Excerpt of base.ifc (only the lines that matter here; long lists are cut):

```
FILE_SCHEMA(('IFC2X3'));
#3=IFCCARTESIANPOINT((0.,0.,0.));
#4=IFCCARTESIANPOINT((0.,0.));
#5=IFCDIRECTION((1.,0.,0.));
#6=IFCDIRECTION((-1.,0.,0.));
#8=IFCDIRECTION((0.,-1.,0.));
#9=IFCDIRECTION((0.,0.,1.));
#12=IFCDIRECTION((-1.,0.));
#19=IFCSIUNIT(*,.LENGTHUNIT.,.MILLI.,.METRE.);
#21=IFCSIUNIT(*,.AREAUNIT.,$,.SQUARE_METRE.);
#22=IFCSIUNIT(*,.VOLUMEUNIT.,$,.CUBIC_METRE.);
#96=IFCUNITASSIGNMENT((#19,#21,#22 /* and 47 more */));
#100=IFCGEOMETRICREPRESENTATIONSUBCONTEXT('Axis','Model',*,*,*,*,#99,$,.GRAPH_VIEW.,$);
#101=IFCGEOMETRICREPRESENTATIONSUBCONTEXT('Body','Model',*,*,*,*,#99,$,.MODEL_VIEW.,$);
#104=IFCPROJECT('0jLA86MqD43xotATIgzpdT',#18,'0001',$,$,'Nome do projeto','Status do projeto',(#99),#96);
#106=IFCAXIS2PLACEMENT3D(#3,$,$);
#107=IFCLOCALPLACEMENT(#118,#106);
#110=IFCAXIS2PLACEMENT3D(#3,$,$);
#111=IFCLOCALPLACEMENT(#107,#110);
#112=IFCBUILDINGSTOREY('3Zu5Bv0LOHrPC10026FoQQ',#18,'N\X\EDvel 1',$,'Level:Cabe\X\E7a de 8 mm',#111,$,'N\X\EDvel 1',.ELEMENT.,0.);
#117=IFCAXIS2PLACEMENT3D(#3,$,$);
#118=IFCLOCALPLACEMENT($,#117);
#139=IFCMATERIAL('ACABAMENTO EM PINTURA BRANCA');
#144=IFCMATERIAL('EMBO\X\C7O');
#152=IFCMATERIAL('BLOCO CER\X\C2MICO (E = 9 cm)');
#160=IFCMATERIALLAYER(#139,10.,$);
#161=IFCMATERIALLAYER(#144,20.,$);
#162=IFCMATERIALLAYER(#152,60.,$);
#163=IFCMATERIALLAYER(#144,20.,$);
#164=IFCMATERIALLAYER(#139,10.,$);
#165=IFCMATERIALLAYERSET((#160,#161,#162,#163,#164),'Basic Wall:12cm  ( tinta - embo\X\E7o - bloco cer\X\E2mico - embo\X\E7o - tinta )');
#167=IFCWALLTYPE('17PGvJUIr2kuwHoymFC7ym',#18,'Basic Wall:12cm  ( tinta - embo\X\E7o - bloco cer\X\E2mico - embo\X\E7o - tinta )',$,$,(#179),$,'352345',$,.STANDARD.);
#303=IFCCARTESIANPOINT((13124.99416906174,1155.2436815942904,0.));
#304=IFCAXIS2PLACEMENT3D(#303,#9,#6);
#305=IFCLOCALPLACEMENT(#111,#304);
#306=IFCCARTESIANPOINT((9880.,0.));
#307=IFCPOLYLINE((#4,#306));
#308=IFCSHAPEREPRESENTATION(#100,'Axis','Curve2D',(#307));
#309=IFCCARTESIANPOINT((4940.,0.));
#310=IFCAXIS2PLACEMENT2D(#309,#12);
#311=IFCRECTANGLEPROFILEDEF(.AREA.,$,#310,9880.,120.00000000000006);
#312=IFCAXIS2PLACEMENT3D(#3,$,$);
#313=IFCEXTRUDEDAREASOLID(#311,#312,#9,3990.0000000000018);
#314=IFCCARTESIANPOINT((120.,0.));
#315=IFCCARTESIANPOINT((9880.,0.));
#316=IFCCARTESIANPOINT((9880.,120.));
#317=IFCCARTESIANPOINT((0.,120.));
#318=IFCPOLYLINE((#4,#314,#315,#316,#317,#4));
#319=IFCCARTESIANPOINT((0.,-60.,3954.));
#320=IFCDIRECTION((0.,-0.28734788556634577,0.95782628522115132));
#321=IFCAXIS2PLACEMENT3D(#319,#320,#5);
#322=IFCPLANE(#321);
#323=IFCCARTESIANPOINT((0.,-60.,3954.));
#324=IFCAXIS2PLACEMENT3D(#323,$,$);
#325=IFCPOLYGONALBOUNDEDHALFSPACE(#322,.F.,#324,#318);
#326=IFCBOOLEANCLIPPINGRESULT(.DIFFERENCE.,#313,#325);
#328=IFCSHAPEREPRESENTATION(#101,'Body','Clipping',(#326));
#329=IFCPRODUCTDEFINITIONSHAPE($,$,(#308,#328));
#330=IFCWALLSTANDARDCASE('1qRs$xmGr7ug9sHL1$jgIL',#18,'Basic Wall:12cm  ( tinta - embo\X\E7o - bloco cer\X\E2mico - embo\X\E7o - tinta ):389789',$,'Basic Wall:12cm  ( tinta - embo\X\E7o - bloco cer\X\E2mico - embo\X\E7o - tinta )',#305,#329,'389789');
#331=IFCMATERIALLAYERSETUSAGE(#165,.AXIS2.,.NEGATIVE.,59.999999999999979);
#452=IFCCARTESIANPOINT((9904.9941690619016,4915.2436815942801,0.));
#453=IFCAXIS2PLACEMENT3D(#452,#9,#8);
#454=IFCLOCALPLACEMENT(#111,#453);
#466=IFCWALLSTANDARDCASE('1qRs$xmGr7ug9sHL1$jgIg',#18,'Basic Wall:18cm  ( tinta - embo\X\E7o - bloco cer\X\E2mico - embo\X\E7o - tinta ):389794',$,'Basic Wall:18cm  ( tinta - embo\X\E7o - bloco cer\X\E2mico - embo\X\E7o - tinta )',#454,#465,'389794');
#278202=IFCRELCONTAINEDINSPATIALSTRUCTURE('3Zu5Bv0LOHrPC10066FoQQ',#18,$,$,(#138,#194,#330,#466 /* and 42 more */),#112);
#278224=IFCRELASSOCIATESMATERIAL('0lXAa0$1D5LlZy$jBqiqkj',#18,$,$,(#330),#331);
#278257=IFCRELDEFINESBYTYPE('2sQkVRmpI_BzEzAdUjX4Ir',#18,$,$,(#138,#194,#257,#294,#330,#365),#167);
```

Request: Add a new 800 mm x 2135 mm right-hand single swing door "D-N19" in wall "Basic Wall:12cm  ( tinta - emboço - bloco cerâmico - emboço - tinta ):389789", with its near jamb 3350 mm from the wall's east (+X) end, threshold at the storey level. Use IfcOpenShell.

```python
import numpy as np
import ifcopenshell
import ifcopenshell.api.feature
import ifcopenshell.api.geometry
import ifcopenshell.api.root
import ifcopenshell.api.spatial
import ifcopenshell.api.type
import ifcopenshell.geom
import ifcopenshell.util.element
import ifcopenshell.util.placement
import ifcopenshell.util.representation
import ifcopenshell.util.shape
import ifcopenshell.util.unit

model = ifcopenshell.open("base.ifc")
unit_scale = ifcopenshell.util.unit.calculate_unit_scale(model)
settings = ifcopenshell.geom.settings()


def volume(element):
    """Net volume in cubic metres, openings subtracted."""
    shape = ifcopenshell.geom.create_shape(settings, element)
    return ifcopenshell.util.shape.get_volume(shape.geometry)


wall = model.by_id(330)
storey = ifcopenshell.util.element.get_container(wall, ifc_class="IfcBuildingStorey")
context = ifcopenshell.util.representation.get_context(model, "Model", "Body", "MODEL_VIEW")
before = volume(wall)

width, height, from_end, sill = 0.8, 2.135, 3.35, 0.0  # metres

# The wall runs along its own X axis, and the end named is its -X end.
wall_shape = ifcopenshell.geom.create_shape(settings, wall)
x, y, z = ifcopenshell.util.shape.get_vertices(wall_shape.geometry).T
start = x.min() + from_end
face, thickness = float(y.min()), float(y.max() - y.min())
wall_matrix = ifcopenshell.util.placement.get_local_placement(wall.ObjectPlacement)
level = ifcopenshell.util.placement.get_local_placement(storey.ObjectPlacement)[2, 3]


def in_wall(x, y):
    """Placement at x, y metres in the wall's axes, at sill height."""
    matrix = wall_matrix.copy()
    matrix[:, 3] = wall_matrix @ np.array([x / unit_scale, y / unit_scale, 0.0, 1.0])
    matrix[2, 3] = level + sill / unit_scale
    return matrix


# Opening: a box that overshoots both wall faces by 50 mm.
opening = ifcopenshell.api.root.create_entity(model, ifc_class="IfcOpeningElement")
box = ifcopenshell.api.geometry.add_wall_representation(
    model, context=context, length=width, height=height, thickness=thickness + 0.1
)
ifcopenshell.api.geometry.assign_representation(model, product=opening, representation=box)
ifcopenshell.api.geometry.edit_object_placement(model, product=opening, matrix=in_wall(start, face - 0.05), is_si=False)
ifcopenshell.api.feature.add_feature(model, feature=opening, element=wall)

door = ifcopenshell.api.root.create_entity(model, ifc_class="IfcDoor", name="D-N19")
door.OverallWidth, door.OverallHeight = width / unit_scale, height / unit_scale
body = ifcopenshell.api.geometry.add_door_representation(
    model,
    context=context,
    overall_width=door.OverallWidth,
    overall_height=door.OverallHeight,
    operation_type="SINGLE_SWING_RIGHT",
    lining_properties={"LiningDepth": thickness / unit_scale, "ThresholdDepth": thickness / unit_scale},
)
ifcopenshell.api.geometry.assign_representation(model, product=door, representation=body)
ifcopenshell.api.spatial.assign_container(model, products=[door], relating_structure=storey)
fills = ifcopenshell.api.feature.add_filling(model, opening=opening, element=door)
fills.OwnerHistory = door.OwnerHistory  # required in IFC2X3

# IFC2X3 keeps the operation on the door style.
style = ifcopenshell.api.root.create_entity(model, ifc_class="IfcDoorStyle", name="D-N19")
style.OperationType, style.ConstructionType = "SINGLE_SWING_RIGHT", "NOTDEFINED"
style.ParameterTakesPrecedence = style.Sizeable = False
ifcopenshell.api.type.assign_type(model, related_objects=[door], relating_type=style)

# The lining spans the wall, so the door starts at the wall face.
ifcopenshell.api.geometry.edit_object_placement(model, product=door, matrix=in_wall(start, face), is_si=False)

after = volume(wall)

print(f"wall volume {before:.3f} -> {after:.3f} m3")

model.write("base_edited.ifc")
```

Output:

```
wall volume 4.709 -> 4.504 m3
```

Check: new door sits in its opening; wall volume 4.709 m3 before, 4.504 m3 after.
